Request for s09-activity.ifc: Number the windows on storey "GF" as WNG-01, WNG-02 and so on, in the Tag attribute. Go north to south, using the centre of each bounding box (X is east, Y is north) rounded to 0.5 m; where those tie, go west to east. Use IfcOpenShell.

First a look at what the model holds.

```python
import ifcopenshell
import ifcopenshell.util.element
import ifcopenshell.util.placement

model = ifcopenshell.open("s09-activity.ifc")
print(model.schema)
storey = next(s for s in model.by_type("IfcBuildingStorey") if s.Name == "GF")
windows = [e for e in ifcopenshell.util.element.get_decomposition(storey) if e.is_a("IfcWindow")]
for e in sorted(windows, key=lambda e: e.id()):
    origin = ifcopenshell.util.placement.get_local_placement(e.ObjectPlacement)[:3, 3]
    print(e.id(), e.Tag, e.Name, origin.round(2) + 0.0, sep=" | ")
```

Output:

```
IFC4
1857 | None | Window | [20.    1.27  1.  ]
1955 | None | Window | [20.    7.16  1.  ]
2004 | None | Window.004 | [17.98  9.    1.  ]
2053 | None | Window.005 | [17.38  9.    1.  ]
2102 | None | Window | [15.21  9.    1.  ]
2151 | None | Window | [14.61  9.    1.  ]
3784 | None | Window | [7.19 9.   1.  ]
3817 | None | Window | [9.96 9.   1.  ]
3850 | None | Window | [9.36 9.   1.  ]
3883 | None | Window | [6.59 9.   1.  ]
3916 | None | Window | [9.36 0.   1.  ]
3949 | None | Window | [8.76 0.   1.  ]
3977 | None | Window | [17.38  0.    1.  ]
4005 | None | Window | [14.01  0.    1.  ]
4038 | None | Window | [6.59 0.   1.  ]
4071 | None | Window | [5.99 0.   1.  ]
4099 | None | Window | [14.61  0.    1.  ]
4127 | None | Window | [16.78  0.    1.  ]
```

```python
import ifcopenshell
import ifcopenshell.geom
import ifcopenshell.util.element
import ifcopenshell.util.shape

model = ifcopenshell.open("s09-activity.ifc")
settings = ifcopenshell.geom.settings()
settings.set("use-world-coords", True)


def centre(element):
    shape = ifcopenshell.geom.create_shape(settings, element)
    return ifcopenshell.util.shape.get_bbox_centroid(shape.geometry)


storey = next(s for s in model.by_type("IfcBuildingStorey") if s.Name == "GF")
windows = [e for e in ifcopenshell.util.element.get_decomposition(storey) if e.is_a("IfcWindow")]

# Insertion points can sit at a corner or the storey origin, so sort by the geometry (in metres).
centres = {e: centre(e) for e in windows}
windows.sort(key=lambda e: (-round(centres[e][1] / 0.5), centres[e][0]))

for i, e in enumerate(windows, start=1):
    number = f"WNG-{i:02d}"
    e.Tag = number
    print(e.id(), number)

model.write("s09-activity_v2.ifc")
```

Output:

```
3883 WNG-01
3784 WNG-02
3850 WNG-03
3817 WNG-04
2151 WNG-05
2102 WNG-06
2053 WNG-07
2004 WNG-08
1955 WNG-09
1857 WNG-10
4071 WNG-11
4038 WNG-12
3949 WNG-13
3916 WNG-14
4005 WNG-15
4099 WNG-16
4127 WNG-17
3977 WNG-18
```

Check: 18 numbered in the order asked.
